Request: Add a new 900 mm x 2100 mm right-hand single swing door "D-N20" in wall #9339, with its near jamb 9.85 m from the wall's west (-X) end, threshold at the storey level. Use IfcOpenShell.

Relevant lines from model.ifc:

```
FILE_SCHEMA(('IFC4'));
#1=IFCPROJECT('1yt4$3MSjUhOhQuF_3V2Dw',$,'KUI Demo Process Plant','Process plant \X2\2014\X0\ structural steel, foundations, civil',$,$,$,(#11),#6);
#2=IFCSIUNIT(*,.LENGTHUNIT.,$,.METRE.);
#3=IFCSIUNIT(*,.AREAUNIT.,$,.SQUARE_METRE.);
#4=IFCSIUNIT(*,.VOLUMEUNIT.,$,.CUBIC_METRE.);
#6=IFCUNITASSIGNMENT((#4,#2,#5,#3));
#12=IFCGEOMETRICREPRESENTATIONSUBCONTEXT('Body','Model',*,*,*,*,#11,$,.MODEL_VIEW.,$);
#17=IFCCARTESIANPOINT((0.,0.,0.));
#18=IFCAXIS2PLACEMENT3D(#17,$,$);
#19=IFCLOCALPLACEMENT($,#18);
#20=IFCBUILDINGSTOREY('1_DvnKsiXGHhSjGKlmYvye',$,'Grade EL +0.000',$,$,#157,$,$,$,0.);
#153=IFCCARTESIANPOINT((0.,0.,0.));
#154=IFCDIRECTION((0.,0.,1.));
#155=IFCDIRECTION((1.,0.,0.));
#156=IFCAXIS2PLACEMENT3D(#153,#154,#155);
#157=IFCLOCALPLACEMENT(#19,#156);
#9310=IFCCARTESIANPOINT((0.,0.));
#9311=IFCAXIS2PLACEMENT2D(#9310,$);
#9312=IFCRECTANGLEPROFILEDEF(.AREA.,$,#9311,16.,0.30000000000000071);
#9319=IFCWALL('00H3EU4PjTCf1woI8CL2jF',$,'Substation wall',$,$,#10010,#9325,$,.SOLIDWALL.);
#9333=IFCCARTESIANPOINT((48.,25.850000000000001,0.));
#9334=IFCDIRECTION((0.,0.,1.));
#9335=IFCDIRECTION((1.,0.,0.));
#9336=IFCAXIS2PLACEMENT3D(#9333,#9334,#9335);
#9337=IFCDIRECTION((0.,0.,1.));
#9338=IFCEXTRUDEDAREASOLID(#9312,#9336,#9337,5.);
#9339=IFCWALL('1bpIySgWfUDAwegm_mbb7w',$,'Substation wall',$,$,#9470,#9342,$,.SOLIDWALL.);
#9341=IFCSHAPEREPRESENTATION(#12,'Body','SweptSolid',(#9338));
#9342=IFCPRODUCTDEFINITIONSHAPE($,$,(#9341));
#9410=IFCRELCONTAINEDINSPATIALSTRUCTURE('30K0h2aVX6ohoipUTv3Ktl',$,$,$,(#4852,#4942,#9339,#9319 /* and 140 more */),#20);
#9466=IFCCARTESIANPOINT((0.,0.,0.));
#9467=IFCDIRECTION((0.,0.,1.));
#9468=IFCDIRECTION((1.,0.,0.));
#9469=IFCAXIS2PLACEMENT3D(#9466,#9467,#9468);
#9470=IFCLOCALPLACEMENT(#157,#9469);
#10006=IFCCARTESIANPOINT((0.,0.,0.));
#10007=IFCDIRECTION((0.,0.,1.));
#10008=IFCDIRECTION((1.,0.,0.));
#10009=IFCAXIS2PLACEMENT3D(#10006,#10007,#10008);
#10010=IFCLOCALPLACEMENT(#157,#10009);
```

```python
import numpy as np
import ifcopenshell
import ifcopenshell.api.feature
import ifcopenshell.api.geometry
import ifcopenshell.api.root
import ifcopenshell.api.spatial
import ifcopenshell.geom
import ifcopenshell.util.element
import ifcopenshell.util.placement
import ifcopenshell.util.representation
import ifcopenshell.util.shape
import ifcopenshell.util.unit

model = ifcopenshell.open("model.ifc")
unit_scale = ifcopenshell.util.unit.calculate_unit_scale(model)
settings = ifcopenshell.geom.settings()


def volume(element):
    """Net volume in cubic metres, openings subtracted."""
    shape = ifcopenshell.geom.create_shape(settings, element)
    return ifcopenshell.util.shape.get_volume(shape.geometry)


wall = model.by_guid("1bpIySgWfUDAwegm_mbb7w")
storey = ifcopenshell.util.element.get_container(wall, ifc_class="IfcBuildingStorey")
context = ifcopenshell.util.representation.get_context(model, "Model", "Body", "MODEL_VIEW")
before = volume(wall)

width, height, from_end, sill = 0.9, 2.1, 9.85, 0.0  # metres

# The wall runs along its own X axis, and the end named is its -X end.
wall_shape = ifcopenshell.geom.create_shape(settings, wall)
x, y, z = ifcopenshell.util.shape.get_vertices(wall_shape.geometry).T
start = x.min() + from_end
face, thickness = float(y.min()), float(y.max() - y.min())
wall_matrix = ifcopenshell.util.placement.get_local_placement(wall.ObjectPlacement)
level = ifcopenshell.util.placement.get_local_placement(storey.ObjectPlacement)[2, 3]


def in_wall(x, y):
    """Placement at x, y metres in the wall's axes, at sill height."""
    matrix = wall_matrix.copy()
    matrix[:, 3] = wall_matrix @ np.array([x / unit_scale, y / unit_scale, 0.0, 1.0])
    matrix[2, 3] = level + sill / unit_scale
    return matrix


# Opening: a box that overshoots both wall faces by 50 mm.
opening = ifcopenshell.api.root.create_entity(model, ifc_class="IfcOpeningElement", predefined_type="OPENING")
box = ifcopenshell.api.geometry.add_wall_representation(
    model, context=context, length=width, height=height, thickness=thickness + 0.1
)
ifcopenshell.api.geometry.assign_representation(model, product=opening, representation=box)
ifcopenshell.api.geometry.edit_object_placement(model, product=opening, matrix=in_wall(start, face - 0.05), is_si=False)
ifcopenshell.api.feature.add_feature(model, feature=opening, element=wall)

door = ifcopenshell.api.root.create_entity(model, ifc_class="IfcDoor", name="D-N20", predefined_type="DOOR")
door.OverallWidth, door.OverallHeight = width / unit_scale, height / unit_scale
door.OperationType = "SINGLE_SWING_RIGHT"
body = ifcopenshell.api.geometry.add_door_representation(
    model,
    context=context,
    overall_width=door.OverallWidth,
    overall_height=door.OverallHeight,
    operation_type="SINGLE_SWING_RIGHT",
    lining_properties={"LiningDepth": thickness / unit_scale, "ThresholdDepth": thickness / unit_scale},
)
ifcopenshell.api.geometry.assign_representation(model, product=door, representation=body)
ifcopenshell.api.spatial.assign_container(model, products=[door], relating_structure=storey)
ifcopenshell.api.feature.add_filling(model, opening=opening, element=door)

# The lining spans the wall, so the door starts at the wall face.
ifcopenshell.api.geometry.edit_object_placement(model, product=door, matrix=in_wall(start, face), is_si=False)

after = volume(wall)

print(f"wall volume {before:.3f} -> {after:.3f} m3")

model.write("model_v2.ifc")
```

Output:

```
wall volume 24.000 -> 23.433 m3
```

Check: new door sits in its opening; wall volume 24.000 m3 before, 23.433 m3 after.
